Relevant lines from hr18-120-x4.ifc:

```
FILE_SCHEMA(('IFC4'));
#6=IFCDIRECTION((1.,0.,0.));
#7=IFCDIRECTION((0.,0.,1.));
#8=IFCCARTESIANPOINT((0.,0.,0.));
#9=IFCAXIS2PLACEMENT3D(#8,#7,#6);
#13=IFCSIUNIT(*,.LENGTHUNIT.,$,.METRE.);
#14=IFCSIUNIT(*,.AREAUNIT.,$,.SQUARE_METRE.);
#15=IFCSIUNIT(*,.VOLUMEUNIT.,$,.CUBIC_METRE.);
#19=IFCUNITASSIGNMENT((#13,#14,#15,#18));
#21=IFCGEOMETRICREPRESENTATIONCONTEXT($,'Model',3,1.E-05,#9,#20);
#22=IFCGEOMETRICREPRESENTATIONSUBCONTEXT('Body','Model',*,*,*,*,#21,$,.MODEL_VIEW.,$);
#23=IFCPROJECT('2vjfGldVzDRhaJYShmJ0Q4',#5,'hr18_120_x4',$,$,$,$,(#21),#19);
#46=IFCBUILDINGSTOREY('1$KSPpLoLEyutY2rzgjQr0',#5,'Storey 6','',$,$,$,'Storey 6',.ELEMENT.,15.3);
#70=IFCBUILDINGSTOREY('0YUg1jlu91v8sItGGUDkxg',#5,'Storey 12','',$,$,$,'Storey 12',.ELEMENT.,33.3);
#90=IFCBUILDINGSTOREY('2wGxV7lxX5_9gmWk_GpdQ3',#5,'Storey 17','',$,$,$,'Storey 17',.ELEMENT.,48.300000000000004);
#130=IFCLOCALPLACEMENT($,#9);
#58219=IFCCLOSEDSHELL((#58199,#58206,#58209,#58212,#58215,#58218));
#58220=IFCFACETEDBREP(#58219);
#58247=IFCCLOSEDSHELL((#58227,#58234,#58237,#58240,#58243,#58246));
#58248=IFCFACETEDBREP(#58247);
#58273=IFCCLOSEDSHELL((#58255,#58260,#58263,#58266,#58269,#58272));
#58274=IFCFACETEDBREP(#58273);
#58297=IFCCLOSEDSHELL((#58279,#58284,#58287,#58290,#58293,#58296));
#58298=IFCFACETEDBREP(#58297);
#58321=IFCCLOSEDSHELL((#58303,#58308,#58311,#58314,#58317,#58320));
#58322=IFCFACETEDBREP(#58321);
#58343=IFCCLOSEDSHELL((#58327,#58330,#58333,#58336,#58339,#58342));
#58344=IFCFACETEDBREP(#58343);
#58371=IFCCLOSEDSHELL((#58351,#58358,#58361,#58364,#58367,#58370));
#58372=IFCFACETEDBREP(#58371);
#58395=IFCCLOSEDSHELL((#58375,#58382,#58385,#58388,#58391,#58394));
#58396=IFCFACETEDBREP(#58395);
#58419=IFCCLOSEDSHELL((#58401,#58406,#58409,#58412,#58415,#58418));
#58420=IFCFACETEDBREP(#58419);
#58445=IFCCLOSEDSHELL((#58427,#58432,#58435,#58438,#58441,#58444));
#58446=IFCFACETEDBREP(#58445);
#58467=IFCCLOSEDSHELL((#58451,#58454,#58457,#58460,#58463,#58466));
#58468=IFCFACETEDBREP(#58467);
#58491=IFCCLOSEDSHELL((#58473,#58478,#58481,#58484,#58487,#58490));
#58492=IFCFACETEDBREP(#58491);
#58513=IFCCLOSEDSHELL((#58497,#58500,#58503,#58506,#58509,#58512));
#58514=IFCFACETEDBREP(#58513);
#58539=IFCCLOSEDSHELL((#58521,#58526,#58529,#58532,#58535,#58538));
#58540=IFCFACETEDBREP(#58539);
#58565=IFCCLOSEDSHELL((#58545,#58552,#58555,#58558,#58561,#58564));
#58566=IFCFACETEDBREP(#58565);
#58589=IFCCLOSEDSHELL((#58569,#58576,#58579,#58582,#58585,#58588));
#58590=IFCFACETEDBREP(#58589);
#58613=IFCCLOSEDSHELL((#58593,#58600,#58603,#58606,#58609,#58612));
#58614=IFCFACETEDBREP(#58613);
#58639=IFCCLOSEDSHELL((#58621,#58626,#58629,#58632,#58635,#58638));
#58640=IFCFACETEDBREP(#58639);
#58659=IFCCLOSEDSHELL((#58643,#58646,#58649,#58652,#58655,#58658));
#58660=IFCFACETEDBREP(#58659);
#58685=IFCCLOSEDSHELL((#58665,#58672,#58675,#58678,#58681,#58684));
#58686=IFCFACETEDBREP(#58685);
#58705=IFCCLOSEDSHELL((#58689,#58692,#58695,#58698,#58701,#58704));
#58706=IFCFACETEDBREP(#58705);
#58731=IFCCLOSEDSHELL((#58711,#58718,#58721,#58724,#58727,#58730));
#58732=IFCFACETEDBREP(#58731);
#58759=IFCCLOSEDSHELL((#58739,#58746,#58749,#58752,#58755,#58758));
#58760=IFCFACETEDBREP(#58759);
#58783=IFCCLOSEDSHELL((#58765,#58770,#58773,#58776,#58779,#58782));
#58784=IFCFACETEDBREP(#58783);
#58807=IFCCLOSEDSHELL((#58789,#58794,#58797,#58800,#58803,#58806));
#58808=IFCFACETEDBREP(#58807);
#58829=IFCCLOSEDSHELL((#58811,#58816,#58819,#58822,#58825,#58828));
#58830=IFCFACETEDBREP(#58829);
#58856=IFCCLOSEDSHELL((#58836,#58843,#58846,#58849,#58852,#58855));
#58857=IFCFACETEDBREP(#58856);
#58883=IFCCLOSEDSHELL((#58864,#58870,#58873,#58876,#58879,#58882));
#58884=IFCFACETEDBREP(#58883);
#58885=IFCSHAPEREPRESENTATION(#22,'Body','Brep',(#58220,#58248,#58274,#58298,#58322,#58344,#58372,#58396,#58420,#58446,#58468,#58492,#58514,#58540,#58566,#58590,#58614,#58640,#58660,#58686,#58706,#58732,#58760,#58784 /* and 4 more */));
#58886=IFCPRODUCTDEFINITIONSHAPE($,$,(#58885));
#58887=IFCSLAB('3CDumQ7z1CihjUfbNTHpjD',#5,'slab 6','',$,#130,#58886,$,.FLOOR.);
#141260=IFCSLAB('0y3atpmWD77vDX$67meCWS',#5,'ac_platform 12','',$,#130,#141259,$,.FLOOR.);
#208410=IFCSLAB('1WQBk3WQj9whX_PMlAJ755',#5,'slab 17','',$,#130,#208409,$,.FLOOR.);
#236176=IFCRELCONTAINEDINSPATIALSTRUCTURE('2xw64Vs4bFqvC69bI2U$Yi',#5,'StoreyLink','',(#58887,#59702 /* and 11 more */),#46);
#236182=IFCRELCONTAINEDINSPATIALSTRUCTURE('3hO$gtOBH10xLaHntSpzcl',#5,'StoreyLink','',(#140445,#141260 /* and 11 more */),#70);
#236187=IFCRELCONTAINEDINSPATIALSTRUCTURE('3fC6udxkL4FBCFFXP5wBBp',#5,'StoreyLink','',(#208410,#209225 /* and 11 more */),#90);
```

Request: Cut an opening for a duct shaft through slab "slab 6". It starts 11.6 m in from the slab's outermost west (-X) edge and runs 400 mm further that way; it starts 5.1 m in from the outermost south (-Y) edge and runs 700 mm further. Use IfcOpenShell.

```python
import numpy as np
import ifcopenshell
import ifcopenshell.api.feature
import ifcopenshell.api.geometry
import ifcopenshell.api.root
import ifcopenshell.geom
import ifcopenshell.util.placement
import ifcopenshell.util.representation
import ifcopenshell.util.shape
import ifcopenshell.util.unit

model = ifcopenshell.open("hr18-120-x4.ifc")
unit_scale = ifcopenshell.util.unit.calculate_unit_scale(model)
settings = ifcopenshell.geom.settings()


def volume(element):
    """Net volume in cubic metres, openings subtracted."""
    shape = ifcopenshell.geom.create_shape(settings, element)
    return ifcopenshell.util.shape.get_volume(shape.geometry)


slab = model.by_id(58887)
before = volume(slab)

# Extent in the slab's own axes, in metres. The edges named are its -X and -Y sides.
slab_shape = ifcopenshell.geom.create_shape(settings, slab)
vertices = ifcopenshell.util.shape.get_vertices(slab_shape.geometry)
x_min, y_min, bottom = vertices.min(axis=0)
top = vertices[:, 2].max()

opening = ifcopenshell.api.root.create_entity(model, ifc_class="IfcOpeningElement", name="Duct shaft opening", predefined_type="OPENING")
context = ifcopenshell.util.representation.get_context(model, "Model", "Body", "MODEL_VIEW")
width, depth = 0.4, 0.7
outline = [(0.0, 0.0), (width, 0.0), (width, depth), (0.0, depth), (0.0, 0.0)]
# Overshoot both faces by 50 mm so the cut is clean.
shape = ifcopenshell.api.geometry.add_slab_representation(
    model, context=context, depth=top - bottom + 0.1, polyline=outline
)
ifcopenshell.api.geometry.assign_representation(model, product=opening, representation=shape)

matrix = ifcopenshell.util.placement.get_local_placement(slab.ObjectPlacement)
matrix[:, 3] = matrix @ np.append(np.array([x_min + 11.6, y_min + 5.1, bottom - 0.05]) / unit_scale, 1.0)
ifcopenshell.api.geometry.edit_object_placement(model, product=opening, matrix=matrix, is_si=False)
ifcopenshell.api.feature.add_feature(model, feature=opening, element=slab)

after = volume(slab)

print(f"slab volume {before:.3f} -> {after:.3f} m3")

model.write("hr18-120-x4_rev.ifc")
```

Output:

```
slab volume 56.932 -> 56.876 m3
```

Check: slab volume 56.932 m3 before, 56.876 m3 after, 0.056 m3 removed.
